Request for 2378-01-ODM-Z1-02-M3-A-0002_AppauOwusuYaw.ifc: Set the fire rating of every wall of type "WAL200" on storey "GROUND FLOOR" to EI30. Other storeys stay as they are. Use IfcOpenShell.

First a look at what the model holds.

```python
import ifcopenshell
import ifcopenshell.util.element

model = ifcopenshell.open("2378-01-ODM-Z1-02-M3-A-0002_AppauOwusuYaw.ifc")
print(model.schema)
storey = next(s for s in model.by_type("IfcBuildingStorey") if s.Name == "GROUND FLOOR")
walls = [e for e in ifcopenshell.util.element.get_decomposition(storey) if e.is_a("IfcWall")]
seen = {}
for e in walls:
    element_type = ifcopenshell.util.element.get_type(e)
    key = (element_type.Name if element_type != e and element_type else None, ifcopenshell.util.element.get_pset(e, "Pset_WallCommon", "FireRating"))
    seen[key] = seen.get(key, 0) + 1
for (name, value), count in sorted(seen.items(), key=str):
    print(count, "x", name, "|", value)
```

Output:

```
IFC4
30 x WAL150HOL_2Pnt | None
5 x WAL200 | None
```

```python
import ifcopenshell
import ifcopenshell.api.pset
import ifcopenshell.util.element

model = ifcopenshell.open("2378-01-ODM-Z1-02-M3-A-0002_AppauOwusuYaw.ifc")

storey = next(s for s in model.by_type("IfcBuildingStorey") if s.Name == "GROUND FLOOR")
walls = [e for e in ifcopenshell.util.element.get_decomposition(storey) if e.is_a("IfcWall")]

count = 0
for e in walls:
    element_type = ifcopenshell.util.element.get_type(e)
    if element_type in (None, e) or element_type.Name != "WAL200":
        continue
    # add_pset returns the element's existing set when there is one.
    pset = ifcopenshell.api.pset.add_pset(model, product=e, name="Pset_WallCommon")
    ifcopenshell.api.pset.edit_pset(model, pset=pset, properties={"FireRating": "EI30"})
    count += 1

print(count, "walls updated")

model.write("2378-01-ODM-Z1-02-M3-A-0002_AppauOwusuYaw-out.ifc")
```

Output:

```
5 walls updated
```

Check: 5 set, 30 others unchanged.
